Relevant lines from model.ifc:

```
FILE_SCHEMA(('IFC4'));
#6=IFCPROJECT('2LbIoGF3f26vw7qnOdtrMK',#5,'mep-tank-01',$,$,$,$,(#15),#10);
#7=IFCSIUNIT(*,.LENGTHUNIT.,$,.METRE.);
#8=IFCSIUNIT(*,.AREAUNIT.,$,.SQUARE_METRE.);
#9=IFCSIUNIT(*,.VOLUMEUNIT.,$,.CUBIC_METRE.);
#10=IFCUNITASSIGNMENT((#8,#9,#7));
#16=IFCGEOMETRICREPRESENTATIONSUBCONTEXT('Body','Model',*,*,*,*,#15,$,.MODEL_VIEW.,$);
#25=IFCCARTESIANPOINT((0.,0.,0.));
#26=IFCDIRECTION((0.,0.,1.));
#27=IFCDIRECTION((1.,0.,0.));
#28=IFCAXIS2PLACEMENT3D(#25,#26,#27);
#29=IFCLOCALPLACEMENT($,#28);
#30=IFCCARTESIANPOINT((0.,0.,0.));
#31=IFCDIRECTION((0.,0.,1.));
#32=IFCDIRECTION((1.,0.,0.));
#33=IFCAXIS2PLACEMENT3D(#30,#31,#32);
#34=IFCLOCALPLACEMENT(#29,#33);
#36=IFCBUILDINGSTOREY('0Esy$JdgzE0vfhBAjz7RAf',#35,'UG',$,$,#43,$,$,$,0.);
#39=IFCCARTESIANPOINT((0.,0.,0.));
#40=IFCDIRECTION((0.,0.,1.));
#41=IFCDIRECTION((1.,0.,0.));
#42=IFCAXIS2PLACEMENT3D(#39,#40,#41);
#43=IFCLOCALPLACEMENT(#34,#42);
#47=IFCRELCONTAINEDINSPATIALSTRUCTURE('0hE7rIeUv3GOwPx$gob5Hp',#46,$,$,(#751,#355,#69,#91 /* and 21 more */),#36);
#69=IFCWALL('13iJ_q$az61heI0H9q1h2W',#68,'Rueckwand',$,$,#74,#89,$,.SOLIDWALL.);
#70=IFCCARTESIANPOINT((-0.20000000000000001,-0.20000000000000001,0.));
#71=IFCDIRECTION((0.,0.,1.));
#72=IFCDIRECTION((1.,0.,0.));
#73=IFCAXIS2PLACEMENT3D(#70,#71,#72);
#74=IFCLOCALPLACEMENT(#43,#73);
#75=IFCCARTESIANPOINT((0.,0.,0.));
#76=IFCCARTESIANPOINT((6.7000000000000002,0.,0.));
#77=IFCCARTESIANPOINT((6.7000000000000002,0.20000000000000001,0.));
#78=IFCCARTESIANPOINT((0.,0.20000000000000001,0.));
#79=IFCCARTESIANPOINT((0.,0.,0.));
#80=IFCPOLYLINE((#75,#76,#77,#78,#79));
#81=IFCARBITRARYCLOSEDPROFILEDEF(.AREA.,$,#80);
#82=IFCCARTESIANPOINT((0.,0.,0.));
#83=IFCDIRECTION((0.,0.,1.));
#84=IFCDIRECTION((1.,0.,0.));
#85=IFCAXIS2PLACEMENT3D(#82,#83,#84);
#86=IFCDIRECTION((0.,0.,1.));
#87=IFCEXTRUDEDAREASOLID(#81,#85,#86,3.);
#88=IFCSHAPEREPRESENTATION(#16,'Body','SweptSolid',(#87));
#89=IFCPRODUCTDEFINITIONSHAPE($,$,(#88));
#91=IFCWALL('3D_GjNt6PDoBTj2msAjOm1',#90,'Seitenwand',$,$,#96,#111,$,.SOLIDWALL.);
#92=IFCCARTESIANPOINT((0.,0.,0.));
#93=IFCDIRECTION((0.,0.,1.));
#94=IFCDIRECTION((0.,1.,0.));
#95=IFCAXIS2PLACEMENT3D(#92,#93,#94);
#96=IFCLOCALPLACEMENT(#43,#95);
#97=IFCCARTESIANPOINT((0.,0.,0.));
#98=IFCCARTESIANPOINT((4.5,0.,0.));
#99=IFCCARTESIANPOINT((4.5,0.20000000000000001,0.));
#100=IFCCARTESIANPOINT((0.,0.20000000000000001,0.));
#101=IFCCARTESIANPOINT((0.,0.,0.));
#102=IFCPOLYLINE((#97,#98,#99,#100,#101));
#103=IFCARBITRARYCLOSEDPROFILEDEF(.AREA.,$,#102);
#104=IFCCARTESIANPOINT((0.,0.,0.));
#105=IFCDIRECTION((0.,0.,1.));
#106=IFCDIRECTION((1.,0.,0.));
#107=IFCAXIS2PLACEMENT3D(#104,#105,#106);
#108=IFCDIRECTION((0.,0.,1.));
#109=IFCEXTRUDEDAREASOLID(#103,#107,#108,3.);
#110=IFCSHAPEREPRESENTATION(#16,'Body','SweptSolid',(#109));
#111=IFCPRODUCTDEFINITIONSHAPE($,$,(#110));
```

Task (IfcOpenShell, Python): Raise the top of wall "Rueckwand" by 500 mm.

```python
import ifcopenshell
import ifcopenshell.geom
import ifcopenshell.util.representation
import ifcopenshell.util.shape
import ifcopenshell.util.unit

model = ifcopenshell.open("model.ifc")
unit_scale = ifcopenshell.util.unit.calculate_unit_scale(model)
settings = ifcopenshell.geom.settings()


def volume(element):
    """Net volume in cubic metres, openings subtracted."""
    shape = ifcopenshell.geom.create_shape(settings, element)
    return ifcopenshell.util.shape.get_volume(shape.geometry)


wall = model.by_guid("13iJ_q$az61heI0H9q1h2W")
before = volume(wall)

body = ifcopenshell.util.representation.get_representation(wall, "Model", "Body")
solid = body.Items[0]
old_height = solid.Depth
solid.Depth += 0.5 / unit_scale
after = volume(wall)

print(f"height {old_height:g} -> {solid.Depth:g}, volume {before:.3f} -> {after:.3f} m3")

model.write("model_v2.ifc")
```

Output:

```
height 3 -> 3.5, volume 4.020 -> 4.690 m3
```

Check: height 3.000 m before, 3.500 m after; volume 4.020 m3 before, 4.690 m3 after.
